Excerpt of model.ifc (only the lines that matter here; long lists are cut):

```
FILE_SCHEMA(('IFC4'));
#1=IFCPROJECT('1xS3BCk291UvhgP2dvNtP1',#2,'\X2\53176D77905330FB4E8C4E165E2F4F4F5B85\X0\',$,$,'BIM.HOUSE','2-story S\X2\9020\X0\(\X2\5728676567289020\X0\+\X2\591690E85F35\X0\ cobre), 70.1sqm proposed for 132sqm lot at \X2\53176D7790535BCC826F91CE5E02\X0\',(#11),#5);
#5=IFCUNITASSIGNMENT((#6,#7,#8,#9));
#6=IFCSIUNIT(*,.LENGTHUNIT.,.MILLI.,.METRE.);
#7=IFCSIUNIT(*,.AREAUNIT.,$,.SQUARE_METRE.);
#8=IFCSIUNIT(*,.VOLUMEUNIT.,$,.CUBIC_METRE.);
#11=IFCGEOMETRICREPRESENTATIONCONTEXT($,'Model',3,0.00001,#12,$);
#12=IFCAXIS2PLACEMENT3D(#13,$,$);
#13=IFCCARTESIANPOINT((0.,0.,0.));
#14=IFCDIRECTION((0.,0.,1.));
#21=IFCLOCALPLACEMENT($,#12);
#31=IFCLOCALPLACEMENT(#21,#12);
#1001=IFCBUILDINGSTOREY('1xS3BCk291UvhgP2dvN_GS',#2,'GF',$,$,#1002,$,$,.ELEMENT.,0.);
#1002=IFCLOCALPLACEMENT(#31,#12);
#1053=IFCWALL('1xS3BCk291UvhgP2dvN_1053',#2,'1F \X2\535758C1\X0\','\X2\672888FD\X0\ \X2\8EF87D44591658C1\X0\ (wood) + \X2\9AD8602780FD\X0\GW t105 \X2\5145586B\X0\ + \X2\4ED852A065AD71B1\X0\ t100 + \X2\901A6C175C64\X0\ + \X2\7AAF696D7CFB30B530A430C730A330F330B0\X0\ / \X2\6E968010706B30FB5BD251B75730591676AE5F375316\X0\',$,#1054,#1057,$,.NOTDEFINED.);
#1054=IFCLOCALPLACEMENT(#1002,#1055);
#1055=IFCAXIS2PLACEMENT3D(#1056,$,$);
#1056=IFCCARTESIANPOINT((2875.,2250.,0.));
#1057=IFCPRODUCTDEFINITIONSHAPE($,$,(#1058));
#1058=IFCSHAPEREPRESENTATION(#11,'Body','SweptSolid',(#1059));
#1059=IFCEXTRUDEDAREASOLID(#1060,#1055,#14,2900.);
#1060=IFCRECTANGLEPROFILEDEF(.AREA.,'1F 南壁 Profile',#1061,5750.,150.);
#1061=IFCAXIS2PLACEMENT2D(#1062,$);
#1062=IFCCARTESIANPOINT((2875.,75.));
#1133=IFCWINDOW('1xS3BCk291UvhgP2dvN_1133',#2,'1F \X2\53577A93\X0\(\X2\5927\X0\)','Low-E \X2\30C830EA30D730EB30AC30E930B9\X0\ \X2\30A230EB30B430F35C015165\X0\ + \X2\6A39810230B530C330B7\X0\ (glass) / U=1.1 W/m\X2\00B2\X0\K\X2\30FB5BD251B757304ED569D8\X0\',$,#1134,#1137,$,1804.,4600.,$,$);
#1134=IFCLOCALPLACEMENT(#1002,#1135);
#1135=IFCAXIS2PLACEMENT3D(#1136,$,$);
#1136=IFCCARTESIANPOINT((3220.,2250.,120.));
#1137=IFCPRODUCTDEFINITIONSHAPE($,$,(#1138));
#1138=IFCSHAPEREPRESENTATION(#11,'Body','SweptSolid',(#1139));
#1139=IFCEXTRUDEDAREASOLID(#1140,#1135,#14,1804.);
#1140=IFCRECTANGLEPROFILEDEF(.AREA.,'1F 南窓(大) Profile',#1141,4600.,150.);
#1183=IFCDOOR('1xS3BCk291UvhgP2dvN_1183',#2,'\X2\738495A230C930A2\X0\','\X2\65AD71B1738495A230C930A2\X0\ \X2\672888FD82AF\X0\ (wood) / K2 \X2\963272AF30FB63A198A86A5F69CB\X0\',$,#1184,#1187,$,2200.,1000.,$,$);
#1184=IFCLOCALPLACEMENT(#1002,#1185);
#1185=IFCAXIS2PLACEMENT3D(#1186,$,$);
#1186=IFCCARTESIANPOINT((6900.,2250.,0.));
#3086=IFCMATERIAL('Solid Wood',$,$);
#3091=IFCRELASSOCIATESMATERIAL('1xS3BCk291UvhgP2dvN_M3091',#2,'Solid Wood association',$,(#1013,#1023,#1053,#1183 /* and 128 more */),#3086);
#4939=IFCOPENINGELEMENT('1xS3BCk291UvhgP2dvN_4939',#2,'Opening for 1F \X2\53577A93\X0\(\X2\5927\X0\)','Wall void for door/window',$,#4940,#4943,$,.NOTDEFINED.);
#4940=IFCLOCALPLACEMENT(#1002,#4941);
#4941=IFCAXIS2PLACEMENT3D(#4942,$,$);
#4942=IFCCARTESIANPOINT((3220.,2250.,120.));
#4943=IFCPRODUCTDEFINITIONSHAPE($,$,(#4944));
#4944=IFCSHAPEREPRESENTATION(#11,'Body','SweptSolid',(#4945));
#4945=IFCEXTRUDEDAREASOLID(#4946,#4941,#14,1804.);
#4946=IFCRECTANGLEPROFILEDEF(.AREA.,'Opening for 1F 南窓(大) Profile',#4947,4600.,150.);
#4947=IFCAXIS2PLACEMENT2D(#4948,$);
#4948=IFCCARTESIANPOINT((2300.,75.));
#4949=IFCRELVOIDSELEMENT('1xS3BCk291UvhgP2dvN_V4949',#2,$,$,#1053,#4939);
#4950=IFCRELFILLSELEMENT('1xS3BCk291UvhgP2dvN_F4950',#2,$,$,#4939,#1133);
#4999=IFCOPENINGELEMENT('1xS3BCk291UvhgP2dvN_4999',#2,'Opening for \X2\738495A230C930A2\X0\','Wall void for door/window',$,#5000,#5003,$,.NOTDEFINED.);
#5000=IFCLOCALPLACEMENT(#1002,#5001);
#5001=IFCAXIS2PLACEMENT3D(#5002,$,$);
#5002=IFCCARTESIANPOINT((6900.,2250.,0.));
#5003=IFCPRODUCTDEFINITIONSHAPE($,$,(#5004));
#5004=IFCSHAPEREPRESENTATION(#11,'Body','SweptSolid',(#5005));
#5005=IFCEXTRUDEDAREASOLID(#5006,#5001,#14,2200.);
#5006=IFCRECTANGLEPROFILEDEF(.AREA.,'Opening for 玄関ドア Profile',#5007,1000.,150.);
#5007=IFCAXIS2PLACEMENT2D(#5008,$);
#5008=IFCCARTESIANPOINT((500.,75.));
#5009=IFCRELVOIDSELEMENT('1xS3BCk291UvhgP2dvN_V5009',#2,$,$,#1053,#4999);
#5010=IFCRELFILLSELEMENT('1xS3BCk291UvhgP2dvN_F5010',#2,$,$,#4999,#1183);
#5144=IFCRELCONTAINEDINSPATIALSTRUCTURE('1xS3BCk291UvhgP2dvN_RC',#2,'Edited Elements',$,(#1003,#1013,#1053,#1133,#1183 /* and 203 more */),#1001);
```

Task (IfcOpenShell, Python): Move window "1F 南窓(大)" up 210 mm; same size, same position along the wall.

```python
import numpy as np
import ifcopenshell
import ifcopenshell.api.geometry
import ifcopenshell.util.placement
import ifcopenshell.util.unit

model = ifcopenshell.open("model.ifc")
unit_scale = ifcopenshell.util.unit.calculate_unit_scale(model)

window = model.by_guid("1xS3BCk291UvhgP2dvN_1133")
opening = window.FillsVoids[0].RelatingOpeningElement
dz = 210.0

shift = np.array([0.0, 0.0, dz])
# The window is not placed relative to its opening, so move both.
for product in (opening, window):
    matrix = ifcopenshell.util.placement.get_local_placement(product.ObjectPlacement)
    matrix[:3, 3] += shift
    ifcopenshell.api.geometry.edit_object_placement(model, product=product, matrix=matrix, is_si=False)

print(f"moved by {dz * unit_scale:+.3f} m")

model.write("model_rev.ifc")
```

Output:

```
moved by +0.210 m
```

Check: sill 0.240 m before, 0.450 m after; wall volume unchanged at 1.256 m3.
